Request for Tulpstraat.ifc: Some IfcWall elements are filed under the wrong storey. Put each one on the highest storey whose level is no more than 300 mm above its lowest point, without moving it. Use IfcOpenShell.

First a look at what the model holds.

```python
import ifcopenshell
import ifcopenshell.util.element
import ifcopenshell.util.placement

model = ifcopenshell.open("Tulpstraat.ifc")
print(model.schema)
for storey in model.by_type("IfcBuildingStorey"):
    level = ifcopenshell.util.placement.get_storey_elevation(storey)
    count = sum(e.is_a("IfcWall") for e in ifcopenshell.util.element.get_contained(storey))
    print(storey.id(), storey.Name, round(level, 3), count, sep=" | ")
```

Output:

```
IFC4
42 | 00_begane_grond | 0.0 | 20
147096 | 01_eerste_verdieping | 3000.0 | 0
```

```python
import ifcopenshell
import ifcopenshell.api.spatial
import ifcopenshell.geom
import ifcopenshell.util.element
import ifcopenshell.util.placement
import ifcopenshell.util.shape
import ifcopenshell.util.unit

model = ifcopenshell.open("Tulpstraat.ifc")
unit_scale = ifcopenshell.util.unit.calculate_unit_scale(model)
settings = ifcopenshell.geom.settings()

levels = sorted(
    ((ifcopenshell.util.placement.get_storey_elevation(s) * unit_scale, s) for s in model.by_type("IfcBuildingStorey")),
    key=lambda pair: pair[0],
)

for e in model.by_type("IfcWall"):
    current = e.ContainedInStructure[0].RelatingStructure if e.ContainedInStructure else None
    if current is None or not current.is_a("IfcBuildingStorey"):
        continue
    shape = ifcopenshell.geom.create_shape(settings, e)
    bottom = ifcopenshell.util.shape.get_shape_bottom_elevation(shape, shape.geometry)
    below = [s for level, s in levels if level <= bottom + 0.3]
    storey = below[-1] if below else levels[0][1]
    if storey != current:
        # assign_container keeps the world position.
        ifcopenshell.api.spatial.assign_container(model, products=[e], relating_structure=storey)
        print(e.id(), current.Name, "->", storey.Name)

model.write("Tulpstraat_rev.ifc")
```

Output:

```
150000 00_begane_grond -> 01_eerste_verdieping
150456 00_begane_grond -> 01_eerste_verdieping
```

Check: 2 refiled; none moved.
